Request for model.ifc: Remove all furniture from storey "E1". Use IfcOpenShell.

First a look at what the model holds.

```python
import ifcopenshell
import ifcopenshell.util.element

model = ifcopenshell.open("model.ifc")
print(model.schema)
storey = next(s for s in model.by_type("IfcBuildingStorey") if s.Name == "E1")
furniture = [e for e in ifcopenshell.util.element.get_decomposition(storey) if e.is_a("IfcFurnishingElement")]
seen = {}
for e in furniture:
    element_type = ifcopenshell.util.element.get_type(e)
    name = element_type.Name if element_type not in (None, e) else None
    seen[name] = seen.get(name, 0) + 1
for name, count in sorted(seen.items(), key=str):
    print(count, "x", name)
```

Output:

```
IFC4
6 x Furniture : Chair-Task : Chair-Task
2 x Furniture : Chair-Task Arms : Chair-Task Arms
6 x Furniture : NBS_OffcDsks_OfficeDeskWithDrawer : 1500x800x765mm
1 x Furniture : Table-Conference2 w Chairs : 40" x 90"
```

```python
import ifcopenshell
import ifcopenshell.api.root
import ifcopenshell.util.element

model = ifcopenshell.open("model.ifc")

storey = next(s for s in model.by_type("IfcBuildingStorey") if s.Name == "E1")
furniture = [e for e in ifcopenshell.util.element.get_decomposition(storey) if e.is_a("IfcFurnishingElement")]

for e in furniture:
    ifcopenshell.api.root.remove_product(model, product=e)
print(len(furniture), "removed")

model.write("model_rev.ifc")
```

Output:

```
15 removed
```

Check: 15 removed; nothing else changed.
